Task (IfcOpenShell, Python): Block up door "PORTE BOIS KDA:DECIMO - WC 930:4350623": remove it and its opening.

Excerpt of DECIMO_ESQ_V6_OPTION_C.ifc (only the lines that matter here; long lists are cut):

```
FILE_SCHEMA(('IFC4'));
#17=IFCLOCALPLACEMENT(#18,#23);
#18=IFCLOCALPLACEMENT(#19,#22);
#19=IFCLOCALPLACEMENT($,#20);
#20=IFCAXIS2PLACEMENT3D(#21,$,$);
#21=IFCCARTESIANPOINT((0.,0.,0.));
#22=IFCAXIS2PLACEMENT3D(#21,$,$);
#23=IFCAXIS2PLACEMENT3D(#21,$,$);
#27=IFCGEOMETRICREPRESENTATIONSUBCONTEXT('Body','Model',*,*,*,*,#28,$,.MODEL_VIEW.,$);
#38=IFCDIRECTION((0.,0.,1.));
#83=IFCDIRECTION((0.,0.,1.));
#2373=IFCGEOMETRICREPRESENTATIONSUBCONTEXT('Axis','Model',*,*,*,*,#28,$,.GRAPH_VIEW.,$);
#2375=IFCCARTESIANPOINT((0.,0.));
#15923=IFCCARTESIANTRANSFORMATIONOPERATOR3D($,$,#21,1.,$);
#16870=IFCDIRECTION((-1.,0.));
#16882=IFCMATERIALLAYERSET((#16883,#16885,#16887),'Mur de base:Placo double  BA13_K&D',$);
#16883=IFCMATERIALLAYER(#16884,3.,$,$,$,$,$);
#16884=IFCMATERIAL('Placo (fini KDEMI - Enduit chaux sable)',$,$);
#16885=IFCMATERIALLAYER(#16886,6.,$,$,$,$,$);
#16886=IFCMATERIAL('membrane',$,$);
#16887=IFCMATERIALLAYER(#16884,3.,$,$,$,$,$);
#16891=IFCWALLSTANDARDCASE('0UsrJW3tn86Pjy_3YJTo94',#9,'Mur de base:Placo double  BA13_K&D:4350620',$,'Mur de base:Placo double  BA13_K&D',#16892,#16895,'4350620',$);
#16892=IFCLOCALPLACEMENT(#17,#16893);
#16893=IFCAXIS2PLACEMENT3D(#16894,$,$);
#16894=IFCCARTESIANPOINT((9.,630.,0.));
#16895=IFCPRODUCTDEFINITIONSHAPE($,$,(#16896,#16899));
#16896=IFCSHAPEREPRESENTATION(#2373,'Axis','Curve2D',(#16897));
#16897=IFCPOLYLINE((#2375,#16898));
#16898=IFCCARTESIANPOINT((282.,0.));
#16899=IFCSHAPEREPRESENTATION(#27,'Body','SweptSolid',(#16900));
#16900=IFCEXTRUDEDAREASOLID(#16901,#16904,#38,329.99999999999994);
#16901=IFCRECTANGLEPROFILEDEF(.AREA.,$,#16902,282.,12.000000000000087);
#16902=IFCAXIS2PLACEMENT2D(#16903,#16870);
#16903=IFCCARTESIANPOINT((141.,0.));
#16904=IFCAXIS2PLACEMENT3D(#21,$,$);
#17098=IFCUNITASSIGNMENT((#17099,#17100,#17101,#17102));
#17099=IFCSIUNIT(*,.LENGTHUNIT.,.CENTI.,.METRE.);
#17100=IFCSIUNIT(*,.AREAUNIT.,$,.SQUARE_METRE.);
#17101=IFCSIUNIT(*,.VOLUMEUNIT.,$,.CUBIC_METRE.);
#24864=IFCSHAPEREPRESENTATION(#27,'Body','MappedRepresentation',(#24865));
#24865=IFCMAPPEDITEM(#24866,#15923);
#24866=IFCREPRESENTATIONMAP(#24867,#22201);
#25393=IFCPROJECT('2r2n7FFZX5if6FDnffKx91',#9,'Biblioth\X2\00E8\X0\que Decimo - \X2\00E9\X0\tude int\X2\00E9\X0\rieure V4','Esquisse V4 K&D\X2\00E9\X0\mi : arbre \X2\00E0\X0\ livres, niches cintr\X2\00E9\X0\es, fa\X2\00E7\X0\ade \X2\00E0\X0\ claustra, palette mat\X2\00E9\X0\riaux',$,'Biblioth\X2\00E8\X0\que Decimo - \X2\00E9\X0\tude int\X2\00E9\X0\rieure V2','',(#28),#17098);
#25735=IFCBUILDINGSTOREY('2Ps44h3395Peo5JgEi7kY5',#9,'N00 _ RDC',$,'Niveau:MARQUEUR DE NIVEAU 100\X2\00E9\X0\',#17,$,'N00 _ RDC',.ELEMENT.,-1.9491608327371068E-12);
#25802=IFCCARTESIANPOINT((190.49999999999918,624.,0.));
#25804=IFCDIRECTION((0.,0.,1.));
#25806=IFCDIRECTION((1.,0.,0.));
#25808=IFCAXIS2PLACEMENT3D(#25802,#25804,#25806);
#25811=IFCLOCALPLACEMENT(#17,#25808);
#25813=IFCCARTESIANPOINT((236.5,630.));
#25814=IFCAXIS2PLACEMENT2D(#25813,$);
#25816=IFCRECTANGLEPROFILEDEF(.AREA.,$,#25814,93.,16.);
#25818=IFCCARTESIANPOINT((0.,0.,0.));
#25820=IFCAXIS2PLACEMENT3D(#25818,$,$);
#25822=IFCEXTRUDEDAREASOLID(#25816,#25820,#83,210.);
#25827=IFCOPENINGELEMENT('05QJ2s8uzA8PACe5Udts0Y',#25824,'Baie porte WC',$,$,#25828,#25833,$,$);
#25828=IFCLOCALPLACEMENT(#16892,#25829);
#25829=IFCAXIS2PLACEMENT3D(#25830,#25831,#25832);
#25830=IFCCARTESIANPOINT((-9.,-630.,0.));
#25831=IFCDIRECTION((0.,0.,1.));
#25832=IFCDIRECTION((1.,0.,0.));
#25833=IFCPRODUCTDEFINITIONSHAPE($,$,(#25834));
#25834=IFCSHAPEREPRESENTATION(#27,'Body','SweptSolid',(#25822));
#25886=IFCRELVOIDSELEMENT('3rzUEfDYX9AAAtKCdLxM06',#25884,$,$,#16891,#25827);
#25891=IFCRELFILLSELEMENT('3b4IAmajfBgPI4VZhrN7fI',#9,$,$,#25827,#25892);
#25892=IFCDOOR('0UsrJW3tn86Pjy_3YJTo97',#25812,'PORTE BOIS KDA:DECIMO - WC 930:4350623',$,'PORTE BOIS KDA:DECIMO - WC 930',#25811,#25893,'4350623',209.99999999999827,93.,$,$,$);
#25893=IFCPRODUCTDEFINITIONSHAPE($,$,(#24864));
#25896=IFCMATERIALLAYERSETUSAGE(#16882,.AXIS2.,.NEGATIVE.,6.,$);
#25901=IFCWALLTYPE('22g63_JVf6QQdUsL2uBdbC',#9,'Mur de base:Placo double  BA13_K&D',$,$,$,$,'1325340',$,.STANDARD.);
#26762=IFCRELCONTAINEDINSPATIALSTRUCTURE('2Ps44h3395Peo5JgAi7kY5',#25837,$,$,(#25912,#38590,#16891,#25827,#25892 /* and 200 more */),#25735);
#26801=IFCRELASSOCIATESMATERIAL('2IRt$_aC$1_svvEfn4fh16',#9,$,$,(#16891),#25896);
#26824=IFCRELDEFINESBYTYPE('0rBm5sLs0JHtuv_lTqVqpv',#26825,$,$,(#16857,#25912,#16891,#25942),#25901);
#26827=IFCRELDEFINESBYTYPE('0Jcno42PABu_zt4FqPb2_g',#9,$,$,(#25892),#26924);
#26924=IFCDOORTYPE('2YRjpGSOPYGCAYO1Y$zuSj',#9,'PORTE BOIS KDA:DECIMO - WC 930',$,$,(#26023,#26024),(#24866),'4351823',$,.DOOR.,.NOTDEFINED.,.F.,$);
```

```python
import ifcopenshell
import ifcopenshell.api.feature
import ifcopenshell.api.root
import ifcopenshell.geom
import ifcopenshell.util.shape

model = ifcopenshell.open("DECIMO_ESQ_V6_OPTION_C.ifc")
settings = ifcopenshell.geom.settings()


def volume(element):
    """Net volume in cubic metres, openings subtracted."""
    shape = ifcopenshell.geom.create_shape(settings, element)
    return ifcopenshell.util.shape.get_volume(shape.geometry)


door = model.by_id(25892)
opening = door.FillsVoids[0].RelatingOpeningElement
wall = opening.VoidsElements[0].RelatingBuildingElement
before = volume(wall)

ifcopenshell.api.root.remove_product(model, product=door)
ifcopenshell.api.feature.remove_feature(model, feature=opening)

after = volume(wall)

print(f"wall volume {before:.3f} -> {after:.3f} m3")

model.write("DECIMO_ESQ_V6_OPTION_C-out.ifc")
```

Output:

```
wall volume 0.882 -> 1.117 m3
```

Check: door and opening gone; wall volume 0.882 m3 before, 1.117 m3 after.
